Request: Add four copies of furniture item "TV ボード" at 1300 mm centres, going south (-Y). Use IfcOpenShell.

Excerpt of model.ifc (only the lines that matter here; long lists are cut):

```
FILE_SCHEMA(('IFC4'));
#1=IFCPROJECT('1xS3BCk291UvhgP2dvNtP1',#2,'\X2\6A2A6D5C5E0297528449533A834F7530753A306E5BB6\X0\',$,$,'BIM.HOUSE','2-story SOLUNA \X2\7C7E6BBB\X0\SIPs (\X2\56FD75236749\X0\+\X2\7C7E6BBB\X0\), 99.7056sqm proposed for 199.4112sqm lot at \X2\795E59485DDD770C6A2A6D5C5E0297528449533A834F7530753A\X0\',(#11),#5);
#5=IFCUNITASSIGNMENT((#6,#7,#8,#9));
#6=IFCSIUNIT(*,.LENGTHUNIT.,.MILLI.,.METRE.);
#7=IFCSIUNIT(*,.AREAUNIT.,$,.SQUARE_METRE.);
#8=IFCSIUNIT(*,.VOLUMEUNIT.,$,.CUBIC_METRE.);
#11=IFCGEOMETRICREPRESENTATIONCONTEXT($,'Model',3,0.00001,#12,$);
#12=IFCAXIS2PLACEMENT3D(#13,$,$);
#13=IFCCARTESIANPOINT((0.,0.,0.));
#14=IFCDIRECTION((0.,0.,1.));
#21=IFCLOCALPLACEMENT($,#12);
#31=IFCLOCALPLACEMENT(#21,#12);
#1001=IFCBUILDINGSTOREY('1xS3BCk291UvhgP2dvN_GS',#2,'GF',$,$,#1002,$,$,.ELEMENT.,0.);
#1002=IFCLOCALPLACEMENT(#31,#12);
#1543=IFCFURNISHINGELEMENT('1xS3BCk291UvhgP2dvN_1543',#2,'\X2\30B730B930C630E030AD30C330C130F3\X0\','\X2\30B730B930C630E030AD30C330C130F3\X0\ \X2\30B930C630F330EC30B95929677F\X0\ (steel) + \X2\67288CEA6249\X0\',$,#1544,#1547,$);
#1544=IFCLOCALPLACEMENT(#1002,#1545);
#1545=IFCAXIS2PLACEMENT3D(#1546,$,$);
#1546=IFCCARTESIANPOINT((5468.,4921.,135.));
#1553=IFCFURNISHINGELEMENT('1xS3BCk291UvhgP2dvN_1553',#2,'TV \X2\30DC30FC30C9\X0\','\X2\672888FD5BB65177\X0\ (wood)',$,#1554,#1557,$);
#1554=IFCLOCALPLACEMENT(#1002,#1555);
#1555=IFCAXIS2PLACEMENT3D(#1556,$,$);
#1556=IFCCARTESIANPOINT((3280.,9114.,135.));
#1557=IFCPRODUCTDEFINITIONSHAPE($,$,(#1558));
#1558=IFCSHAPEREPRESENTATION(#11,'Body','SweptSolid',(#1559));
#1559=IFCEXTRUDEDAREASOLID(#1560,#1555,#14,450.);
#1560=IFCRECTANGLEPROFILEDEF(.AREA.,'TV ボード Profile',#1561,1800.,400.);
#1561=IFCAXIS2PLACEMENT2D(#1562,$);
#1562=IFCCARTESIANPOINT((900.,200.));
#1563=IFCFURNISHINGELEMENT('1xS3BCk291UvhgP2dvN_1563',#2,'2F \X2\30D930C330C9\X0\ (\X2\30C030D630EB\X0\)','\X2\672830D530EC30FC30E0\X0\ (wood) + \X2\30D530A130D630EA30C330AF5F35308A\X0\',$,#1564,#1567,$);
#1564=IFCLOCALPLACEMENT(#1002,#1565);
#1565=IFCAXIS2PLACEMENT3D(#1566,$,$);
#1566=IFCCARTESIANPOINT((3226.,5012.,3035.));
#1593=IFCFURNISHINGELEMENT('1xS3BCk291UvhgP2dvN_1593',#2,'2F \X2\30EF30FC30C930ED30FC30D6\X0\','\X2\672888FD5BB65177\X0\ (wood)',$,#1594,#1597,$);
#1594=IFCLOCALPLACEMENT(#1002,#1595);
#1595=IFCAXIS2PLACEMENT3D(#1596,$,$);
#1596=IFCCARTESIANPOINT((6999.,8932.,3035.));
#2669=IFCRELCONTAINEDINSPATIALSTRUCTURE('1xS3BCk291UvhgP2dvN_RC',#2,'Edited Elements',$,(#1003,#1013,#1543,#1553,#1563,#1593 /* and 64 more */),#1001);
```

```python
import numpy as np
import ifcopenshell
import ifcopenshell.api.geometry
import ifcopenshell.api.root
import ifcopenshell.util.element
import ifcopenshell.util.placement
import ifcopenshell.util.unit

model = ifcopenshell.open("model.ifc")
unit_scale = ifcopenshell.util.unit.calculate_unit_scale(model)


def reuse_history(source, copy):
    """copy_class also copies each property set's owner history, people and application; keep the originals."""
    for rel in copy.IsDefinedBy:
        if rel.is_a("IfcRelDefinesByProperties") and (history := rel.RelatingPropertyDefinition.OwnerHistory):
            rel.RelatingPropertyDefinition.OwnerHistory = source.OwnerHistory
            ifcopenshell.util.element.remove_deep2(model, history)


source = model.by_guid("1xS3BCk291UvhgP2dvN_1553")
base = ifcopenshell.util.placement.get_local_placement(source.ObjectPlacement)
step = np.array([0.0, -1.0, 0.0]) * 1.3 / unit_scale

for i in range(1, 5):
    copy = ifcopenshell.api.root.copy_class(model, product=source)
    copy.Representation = ifcopenshell.util.element.copy_deep(
        model, source.Representation, exclude=["IfcGeometricRepresentationContext", "IfcRepresentationMap"]
    )
    reuse_history(source, copy)
    matrix = base.copy()
    matrix[:3, 3] += i * step
    print("added at", matrix[:3, 3].round(3) + 0.0)
    ifcopenshell.api.geometry.edit_object_placement(model, product=copy, matrix=matrix, is_si=False)

model.write("model_updated.ifc")
```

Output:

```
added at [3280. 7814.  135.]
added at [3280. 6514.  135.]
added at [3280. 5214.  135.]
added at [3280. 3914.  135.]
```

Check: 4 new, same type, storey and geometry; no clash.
